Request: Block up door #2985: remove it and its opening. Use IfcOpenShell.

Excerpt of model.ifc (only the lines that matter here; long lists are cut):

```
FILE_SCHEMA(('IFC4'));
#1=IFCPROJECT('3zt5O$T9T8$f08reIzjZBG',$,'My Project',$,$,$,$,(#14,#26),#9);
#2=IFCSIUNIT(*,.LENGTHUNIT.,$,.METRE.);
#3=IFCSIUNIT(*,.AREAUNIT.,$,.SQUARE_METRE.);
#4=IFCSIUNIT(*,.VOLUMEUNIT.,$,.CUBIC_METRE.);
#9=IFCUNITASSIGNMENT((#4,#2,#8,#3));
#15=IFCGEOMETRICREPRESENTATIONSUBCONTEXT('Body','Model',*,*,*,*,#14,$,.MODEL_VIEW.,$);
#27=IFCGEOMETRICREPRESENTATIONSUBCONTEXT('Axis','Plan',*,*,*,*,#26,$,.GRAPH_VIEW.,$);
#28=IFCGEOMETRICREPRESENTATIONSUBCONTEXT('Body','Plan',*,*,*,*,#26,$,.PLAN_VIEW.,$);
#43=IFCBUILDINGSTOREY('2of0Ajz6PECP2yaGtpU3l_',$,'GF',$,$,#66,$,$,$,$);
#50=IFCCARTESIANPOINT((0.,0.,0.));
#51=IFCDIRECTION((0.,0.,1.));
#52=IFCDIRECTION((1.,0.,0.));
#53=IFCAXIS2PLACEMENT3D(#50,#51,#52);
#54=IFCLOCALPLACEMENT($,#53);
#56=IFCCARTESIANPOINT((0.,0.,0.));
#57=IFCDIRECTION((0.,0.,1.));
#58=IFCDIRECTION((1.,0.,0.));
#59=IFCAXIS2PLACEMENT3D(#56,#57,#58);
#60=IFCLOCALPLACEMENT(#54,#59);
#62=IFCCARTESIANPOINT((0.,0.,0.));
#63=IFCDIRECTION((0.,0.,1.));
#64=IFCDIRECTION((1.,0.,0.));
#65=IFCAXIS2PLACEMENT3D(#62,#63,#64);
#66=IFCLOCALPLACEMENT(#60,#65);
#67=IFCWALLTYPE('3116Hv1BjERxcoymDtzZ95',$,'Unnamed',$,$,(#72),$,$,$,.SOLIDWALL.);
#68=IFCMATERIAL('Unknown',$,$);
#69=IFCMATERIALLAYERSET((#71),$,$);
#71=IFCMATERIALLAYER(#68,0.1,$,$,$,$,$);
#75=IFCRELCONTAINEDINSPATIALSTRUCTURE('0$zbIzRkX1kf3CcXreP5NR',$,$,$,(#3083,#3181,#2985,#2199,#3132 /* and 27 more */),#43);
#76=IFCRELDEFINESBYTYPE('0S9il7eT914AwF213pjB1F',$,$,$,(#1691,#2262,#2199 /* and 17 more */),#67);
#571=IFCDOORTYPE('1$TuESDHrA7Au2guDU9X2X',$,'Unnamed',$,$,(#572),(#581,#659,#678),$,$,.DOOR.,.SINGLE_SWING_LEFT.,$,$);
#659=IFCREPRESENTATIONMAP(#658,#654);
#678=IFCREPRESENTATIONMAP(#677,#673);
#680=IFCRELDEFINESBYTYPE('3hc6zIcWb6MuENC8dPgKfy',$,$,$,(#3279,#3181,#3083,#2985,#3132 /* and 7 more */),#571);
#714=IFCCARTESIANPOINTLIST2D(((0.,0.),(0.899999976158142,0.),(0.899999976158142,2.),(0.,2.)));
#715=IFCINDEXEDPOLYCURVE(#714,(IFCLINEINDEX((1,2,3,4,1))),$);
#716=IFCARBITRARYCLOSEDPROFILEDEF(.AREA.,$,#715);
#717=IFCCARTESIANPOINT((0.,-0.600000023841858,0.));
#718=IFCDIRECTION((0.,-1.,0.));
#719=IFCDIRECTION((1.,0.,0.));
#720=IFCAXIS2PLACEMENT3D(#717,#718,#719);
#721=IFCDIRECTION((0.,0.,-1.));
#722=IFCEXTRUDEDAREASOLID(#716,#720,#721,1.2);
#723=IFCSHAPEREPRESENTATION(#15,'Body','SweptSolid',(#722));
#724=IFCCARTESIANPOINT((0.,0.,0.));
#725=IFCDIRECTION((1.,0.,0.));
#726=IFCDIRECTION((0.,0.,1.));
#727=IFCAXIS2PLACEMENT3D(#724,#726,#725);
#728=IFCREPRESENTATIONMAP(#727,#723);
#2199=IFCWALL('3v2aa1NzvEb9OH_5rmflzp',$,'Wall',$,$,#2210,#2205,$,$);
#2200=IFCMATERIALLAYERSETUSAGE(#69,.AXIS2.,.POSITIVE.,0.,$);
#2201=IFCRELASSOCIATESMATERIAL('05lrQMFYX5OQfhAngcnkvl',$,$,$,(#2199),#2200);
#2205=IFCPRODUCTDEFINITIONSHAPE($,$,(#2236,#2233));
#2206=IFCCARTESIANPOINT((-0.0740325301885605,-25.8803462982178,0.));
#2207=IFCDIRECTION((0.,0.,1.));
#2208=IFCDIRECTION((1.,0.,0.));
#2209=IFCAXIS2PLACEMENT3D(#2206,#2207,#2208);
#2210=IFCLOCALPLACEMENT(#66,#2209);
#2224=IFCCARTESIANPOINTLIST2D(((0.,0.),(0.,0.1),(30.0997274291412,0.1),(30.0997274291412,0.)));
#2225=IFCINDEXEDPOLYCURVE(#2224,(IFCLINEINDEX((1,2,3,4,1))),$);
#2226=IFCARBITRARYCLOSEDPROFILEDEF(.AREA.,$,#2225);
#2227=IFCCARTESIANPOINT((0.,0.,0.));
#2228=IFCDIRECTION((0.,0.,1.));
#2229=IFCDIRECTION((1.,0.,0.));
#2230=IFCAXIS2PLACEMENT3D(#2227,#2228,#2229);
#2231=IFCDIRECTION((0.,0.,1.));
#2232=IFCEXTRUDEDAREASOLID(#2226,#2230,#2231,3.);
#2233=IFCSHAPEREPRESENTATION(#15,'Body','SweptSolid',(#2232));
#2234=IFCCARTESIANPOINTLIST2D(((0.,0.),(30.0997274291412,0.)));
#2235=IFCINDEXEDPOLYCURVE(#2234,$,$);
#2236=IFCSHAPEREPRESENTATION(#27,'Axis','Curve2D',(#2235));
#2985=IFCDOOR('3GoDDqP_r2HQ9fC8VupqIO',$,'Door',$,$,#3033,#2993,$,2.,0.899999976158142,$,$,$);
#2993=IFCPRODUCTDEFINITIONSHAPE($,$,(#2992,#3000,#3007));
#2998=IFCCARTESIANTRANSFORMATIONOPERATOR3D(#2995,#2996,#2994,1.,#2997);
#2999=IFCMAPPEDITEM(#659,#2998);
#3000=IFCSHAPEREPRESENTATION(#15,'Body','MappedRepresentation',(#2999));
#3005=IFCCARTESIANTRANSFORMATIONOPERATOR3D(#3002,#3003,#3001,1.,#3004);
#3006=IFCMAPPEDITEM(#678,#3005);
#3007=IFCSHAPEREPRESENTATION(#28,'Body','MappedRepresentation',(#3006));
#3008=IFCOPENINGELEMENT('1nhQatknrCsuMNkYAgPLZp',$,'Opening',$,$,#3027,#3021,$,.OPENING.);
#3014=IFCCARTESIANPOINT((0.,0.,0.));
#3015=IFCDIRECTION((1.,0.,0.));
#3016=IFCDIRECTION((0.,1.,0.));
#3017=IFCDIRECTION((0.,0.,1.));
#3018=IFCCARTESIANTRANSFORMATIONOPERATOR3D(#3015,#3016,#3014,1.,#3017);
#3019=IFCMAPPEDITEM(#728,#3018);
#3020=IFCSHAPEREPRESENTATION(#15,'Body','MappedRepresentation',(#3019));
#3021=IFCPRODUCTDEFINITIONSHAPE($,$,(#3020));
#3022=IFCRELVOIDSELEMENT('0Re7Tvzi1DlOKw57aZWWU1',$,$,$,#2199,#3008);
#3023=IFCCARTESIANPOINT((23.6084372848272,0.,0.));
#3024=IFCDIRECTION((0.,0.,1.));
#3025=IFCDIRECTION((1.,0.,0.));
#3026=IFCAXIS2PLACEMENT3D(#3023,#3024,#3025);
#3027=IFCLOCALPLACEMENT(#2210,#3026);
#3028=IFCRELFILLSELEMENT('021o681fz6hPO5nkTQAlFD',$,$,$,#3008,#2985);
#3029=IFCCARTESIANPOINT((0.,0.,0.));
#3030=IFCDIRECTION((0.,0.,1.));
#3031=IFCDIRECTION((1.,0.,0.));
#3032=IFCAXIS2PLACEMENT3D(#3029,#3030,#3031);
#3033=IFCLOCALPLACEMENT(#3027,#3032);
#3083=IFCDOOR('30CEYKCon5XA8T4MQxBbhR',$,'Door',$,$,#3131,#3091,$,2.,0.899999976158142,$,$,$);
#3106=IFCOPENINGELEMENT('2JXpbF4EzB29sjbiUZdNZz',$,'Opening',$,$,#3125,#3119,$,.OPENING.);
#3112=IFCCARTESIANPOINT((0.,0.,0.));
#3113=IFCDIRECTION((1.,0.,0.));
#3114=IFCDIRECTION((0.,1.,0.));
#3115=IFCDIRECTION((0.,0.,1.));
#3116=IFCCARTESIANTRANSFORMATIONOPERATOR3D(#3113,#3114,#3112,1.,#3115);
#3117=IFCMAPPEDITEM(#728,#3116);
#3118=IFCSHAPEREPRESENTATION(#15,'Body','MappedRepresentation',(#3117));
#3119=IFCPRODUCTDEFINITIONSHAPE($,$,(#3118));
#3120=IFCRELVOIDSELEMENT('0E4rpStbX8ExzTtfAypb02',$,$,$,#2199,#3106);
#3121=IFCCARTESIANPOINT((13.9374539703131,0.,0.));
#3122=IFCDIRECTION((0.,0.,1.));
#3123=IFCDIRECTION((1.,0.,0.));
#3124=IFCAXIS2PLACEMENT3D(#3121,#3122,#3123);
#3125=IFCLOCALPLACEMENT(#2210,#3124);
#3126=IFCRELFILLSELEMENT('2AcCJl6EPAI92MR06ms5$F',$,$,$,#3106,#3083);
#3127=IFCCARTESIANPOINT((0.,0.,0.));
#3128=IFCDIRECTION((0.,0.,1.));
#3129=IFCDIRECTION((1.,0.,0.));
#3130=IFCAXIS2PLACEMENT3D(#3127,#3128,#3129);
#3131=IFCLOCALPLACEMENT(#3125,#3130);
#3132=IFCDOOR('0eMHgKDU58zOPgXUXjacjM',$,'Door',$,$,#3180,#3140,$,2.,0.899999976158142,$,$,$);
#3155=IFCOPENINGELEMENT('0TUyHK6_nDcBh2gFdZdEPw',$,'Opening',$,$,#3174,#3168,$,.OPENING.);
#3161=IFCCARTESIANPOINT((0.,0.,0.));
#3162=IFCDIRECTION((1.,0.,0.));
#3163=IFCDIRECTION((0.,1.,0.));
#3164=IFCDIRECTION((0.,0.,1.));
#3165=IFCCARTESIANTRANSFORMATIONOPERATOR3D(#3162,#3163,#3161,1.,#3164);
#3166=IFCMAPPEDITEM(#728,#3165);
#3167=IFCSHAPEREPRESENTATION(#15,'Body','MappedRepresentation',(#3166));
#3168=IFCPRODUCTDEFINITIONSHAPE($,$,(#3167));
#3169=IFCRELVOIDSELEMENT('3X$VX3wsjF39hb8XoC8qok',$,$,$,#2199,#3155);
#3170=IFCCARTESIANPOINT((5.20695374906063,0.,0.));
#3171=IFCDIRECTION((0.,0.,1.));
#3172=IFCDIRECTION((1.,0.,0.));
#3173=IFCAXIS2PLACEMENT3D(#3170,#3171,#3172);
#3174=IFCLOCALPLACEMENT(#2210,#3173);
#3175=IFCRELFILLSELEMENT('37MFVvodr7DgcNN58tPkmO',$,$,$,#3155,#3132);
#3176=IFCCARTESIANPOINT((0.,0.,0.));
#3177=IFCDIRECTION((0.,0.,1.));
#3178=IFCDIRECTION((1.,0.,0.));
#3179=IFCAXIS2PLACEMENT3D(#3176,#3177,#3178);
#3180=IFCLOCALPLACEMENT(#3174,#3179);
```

```python
import ifcopenshell
import ifcopenshell.api.feature
import ifcopenshell.api.root
import ifcopenshell.geom
import ifcopenshell.util.shape

model = ifcopenshell.open("model.ifc")
settings = ifcopenshell.geom.settings()


def volume(element):
    """Net volume in cubic metres, openings subtracted."""
    shape = ifcopenshell.geom.create_shape(settings, element)
    return ifcopenshell.util.shape.get_volume(shape.geometry)


door = model.by_guid("3GoDDqP_r2HQ9fC8VupqIO")
opening = door.FillsVoids[0].RelatingOpeningElement
wall = opening.VoidsElements[0].RelatingBuildingElement
before = volume(wall)

ifcopenshell.api.root.remove_product(model, product=door)
ifcopenshell.api.feature.remove_feature(model, feature=opening)

after = volume(wall)

print(f"wall volume {before:.3f} -> {after:.3f} m3")

model.write("model_v2.ifc")
```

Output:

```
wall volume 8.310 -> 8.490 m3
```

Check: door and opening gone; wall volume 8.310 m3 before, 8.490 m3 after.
